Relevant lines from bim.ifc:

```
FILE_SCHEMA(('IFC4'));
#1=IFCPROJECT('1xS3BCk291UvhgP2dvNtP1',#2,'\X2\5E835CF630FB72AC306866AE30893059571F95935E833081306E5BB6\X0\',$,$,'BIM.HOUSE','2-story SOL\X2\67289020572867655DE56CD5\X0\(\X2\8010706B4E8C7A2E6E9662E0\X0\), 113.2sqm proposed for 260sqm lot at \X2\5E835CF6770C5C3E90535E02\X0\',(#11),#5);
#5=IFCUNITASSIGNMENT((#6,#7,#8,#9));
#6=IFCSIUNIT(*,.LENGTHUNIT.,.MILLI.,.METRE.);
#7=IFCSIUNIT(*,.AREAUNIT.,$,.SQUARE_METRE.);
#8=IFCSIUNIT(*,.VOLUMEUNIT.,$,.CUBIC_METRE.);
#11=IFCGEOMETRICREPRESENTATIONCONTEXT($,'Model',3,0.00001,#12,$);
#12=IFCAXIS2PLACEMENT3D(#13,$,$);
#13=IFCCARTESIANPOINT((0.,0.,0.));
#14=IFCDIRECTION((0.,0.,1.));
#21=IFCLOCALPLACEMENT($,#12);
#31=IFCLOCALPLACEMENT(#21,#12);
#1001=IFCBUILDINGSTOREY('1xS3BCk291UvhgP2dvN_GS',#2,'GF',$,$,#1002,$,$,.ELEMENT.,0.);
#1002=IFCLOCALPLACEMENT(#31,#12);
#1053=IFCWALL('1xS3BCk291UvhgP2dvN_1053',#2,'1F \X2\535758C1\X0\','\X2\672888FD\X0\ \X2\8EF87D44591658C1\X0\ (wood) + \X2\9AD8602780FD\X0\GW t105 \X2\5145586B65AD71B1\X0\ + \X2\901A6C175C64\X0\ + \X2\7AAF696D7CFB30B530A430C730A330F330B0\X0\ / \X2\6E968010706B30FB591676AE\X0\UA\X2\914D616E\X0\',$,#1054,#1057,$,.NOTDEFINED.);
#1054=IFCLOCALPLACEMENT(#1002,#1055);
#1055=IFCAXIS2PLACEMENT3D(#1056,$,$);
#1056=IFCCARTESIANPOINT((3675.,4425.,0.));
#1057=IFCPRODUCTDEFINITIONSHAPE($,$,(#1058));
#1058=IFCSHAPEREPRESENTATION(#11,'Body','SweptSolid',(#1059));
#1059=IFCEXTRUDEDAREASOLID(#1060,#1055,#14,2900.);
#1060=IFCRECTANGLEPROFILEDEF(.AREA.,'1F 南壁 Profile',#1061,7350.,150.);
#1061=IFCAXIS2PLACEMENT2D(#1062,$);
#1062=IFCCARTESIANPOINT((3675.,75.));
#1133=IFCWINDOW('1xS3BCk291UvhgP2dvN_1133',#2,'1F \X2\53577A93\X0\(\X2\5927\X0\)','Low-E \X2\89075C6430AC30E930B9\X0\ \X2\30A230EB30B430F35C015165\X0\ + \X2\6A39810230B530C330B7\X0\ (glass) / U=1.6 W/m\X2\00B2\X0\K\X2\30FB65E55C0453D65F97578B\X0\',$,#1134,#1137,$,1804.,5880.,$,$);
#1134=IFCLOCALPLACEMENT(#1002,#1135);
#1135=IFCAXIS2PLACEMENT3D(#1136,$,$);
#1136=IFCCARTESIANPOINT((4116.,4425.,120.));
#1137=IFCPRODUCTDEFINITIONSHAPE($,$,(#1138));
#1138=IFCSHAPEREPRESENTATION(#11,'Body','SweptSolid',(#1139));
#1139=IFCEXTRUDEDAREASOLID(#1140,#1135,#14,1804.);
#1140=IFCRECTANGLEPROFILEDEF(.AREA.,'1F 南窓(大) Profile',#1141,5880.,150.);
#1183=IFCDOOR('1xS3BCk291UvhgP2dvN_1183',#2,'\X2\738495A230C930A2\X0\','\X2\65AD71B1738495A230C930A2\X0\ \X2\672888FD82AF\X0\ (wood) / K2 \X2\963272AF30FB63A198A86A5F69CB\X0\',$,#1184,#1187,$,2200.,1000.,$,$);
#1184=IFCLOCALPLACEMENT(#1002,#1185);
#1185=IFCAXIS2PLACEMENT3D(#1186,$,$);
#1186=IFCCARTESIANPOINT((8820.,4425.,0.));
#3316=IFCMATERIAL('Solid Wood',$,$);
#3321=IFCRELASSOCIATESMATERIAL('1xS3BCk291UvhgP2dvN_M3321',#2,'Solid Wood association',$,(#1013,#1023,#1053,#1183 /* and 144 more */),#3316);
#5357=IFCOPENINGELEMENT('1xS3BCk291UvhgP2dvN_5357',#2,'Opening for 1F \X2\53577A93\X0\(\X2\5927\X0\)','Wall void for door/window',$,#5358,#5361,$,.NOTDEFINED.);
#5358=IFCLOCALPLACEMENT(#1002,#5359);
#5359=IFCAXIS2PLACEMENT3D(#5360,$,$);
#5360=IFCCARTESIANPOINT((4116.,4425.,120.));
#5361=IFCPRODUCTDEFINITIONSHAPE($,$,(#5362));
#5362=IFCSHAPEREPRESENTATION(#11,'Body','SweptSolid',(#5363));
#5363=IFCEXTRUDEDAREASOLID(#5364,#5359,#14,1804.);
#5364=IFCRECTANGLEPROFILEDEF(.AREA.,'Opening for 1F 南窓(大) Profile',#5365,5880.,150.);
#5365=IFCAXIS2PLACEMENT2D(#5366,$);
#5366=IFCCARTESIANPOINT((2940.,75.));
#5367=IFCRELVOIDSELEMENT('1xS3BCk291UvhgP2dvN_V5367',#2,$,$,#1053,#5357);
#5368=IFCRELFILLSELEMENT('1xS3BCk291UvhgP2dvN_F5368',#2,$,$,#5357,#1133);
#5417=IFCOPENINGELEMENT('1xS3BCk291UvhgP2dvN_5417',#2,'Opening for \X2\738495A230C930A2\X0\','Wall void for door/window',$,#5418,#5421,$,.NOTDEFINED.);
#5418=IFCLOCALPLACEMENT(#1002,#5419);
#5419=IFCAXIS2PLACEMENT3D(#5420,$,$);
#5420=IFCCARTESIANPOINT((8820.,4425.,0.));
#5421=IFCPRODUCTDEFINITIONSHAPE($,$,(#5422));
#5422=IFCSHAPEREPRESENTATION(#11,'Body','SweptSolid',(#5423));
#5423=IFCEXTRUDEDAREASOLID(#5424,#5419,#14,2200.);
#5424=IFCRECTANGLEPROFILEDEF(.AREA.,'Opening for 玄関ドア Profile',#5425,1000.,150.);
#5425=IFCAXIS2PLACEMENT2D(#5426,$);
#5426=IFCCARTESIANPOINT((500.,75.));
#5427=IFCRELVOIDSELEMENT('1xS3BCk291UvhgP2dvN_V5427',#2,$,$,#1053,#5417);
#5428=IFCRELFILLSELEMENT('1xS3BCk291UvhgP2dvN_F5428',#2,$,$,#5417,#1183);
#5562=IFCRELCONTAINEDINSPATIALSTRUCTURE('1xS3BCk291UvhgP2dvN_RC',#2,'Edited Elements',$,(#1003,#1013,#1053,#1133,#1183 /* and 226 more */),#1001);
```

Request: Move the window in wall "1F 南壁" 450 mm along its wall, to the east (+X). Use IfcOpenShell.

```python
import ifcopenshell
import ifcopenshell.api.geometry
import ifcopenshell.util.placement
import ifcopenshell.util.unit

model = ifcopenshell.open("bim.ifc")
unit_scale = ifcopenshell.util.unit.calculate_unit_scale(model)

window = model.by_guid("1xS3BCk291UvhgP2dvN_1133")
opening = window.FillsVoids[0].RelatingOpeningElement
wall = opening.VoidsElements[0].RelatingBuildingElement

wall_matrix = ifcopenshell.util.placement.get_local_placement(wall.ObjectPlacement)
shift = wall_matrix[:3, 0] * 0.45 / unit_scale
before = ifcopenshell.util.placement.get_local_placement(window.ObjectPlacement)[:3, 3].copy()

# The window is not placed relative to its opening, so move both.
for product in (opening, window):
    matrix = ifcopenshell.util.placement.get_local_placement(product.ObjectPlacement)
    matrix[:3, 3] += shift
    ifcopenshell.api.geometry.edit_object_placement(model, product=product, matrix=matrix, is_si=False)

after = ifcopenshell.util.placement.get_local_placement(window.ObjectPlacement)[:3, 3]
print("window moved by", (after - before).round(3) + 0.0)

model.write("bim-out.ifc")
```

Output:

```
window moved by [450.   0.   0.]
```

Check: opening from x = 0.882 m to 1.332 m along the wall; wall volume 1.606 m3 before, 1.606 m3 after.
